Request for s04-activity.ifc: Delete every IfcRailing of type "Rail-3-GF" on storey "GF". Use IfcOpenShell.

First a look at what the model holds.

```python
import ifcopenshell
import ifcopenshell.util.element

model = ifcopenshell.open("s04-activity.ifc")
print(model.schema)
storey = next(s for s in model.by_type("IfcBuildingStorey") if s.Name == "GF")
railings = [e for e in ifcopenshell.util.element.get_decomposition(storey) if e.is_a("IfcRailing")]
seen = {}
for e in railings:
    element_type = ifcopenshell.util.element.get_type(e)
    name = element_type.Name if element_type not in (None, e) else None
    seen[name] = seen.get(name, 0) + 1
for name, count in sorted(seen.items(), key=str):
    print(count, "x", name)
```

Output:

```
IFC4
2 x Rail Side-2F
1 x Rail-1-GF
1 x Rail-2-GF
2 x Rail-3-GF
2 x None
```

```python
import ifcopenshell
import ifcopenshell.api.root
import ifcopenshell.util.element

model = ifcopenshell.open("s04-activity.ifc")

storey = next(s for s in model.by_type("IfcBuildingStorey") if s.Name == "GF")
railings = [e for e in ifcopenshell.util.element.get_decomposition(storey) if e.is_a("IfcRailing")]
targets = [e for e in railings if (t := ifcopenshell.util.element.get_type(e)) not in (None, e) and t.Name == "Rail-3-GF"]

for e in targets:
    ifcopenshell.api.root.remove_product(model, product=e)
print(len(targets), "removed")

model.write("s04-activity_rev.ifc")
```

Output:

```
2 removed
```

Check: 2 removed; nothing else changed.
